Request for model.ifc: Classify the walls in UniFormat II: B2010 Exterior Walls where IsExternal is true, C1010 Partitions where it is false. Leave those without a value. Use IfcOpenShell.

First a look at what the model holds.

```python
import ifcopenshell
import ifcopenshell.util.element

model = ifcopenshell.open("model.ifc")
print(model.schema)
print("classifications:", [c.Name for c in model.by_type("IfcClassification")])
values = [ifcopenshell.util.element.get_pset(e, "Pset_WallCommon", "IsExternal") for e in model.by_type("IfcWall")]
for value in (True, False, None):
    print("IsExternal", value, values.count(value))
```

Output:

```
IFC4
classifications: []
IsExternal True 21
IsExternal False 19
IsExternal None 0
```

```python
import ifcopenshell
import ifcopenshell.api.classification
import ifcopenshell.util.element

model = ifcopenshell.open("model.ifc")

system = ifcopenshell.api.classification.add_classification(model, classification="UniFormat II")

walls = model.by_type("IfcWall")
external = {e: ifcopenshell.util.element.get_pset(e, "Pset_WallCommon", "IsExternal") for e in walls}
for flag, code, name in ((True, "B2010", "Exterior Walls"), (False, "C1010", "Partitions")):
    products = [e for e in walls if external[e] is flag]
    ifcopenshell.api.classification.add_reference(
        model, products=products, classification=system, identification=code, name=name
    )
    print(code, len(products))

model.write("model_v2.ifc")
```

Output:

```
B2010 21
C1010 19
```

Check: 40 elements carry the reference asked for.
